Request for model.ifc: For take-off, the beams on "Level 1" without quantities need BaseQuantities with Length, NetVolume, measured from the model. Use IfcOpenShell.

First a look at what the model holds.

```python
import ifcopenshell
import ifcopenshell.util.element
import ifcopenshell.util.unit

model = ifcopenshell.open("model.ifc")
print(model.schema)
for unit_type in ("LENGTHUNIT", "AREAUNIT", "VOLUMEUNIT"):
    print(unit_type, ifcopenshell.util.unit.calculate_unit_scale(model, unit_type))
storey = next(s for s in model.by_type("IfcBuildingStorey") if s.Name == "Level 1")
beams = [e for e in ifcopenshell.util.element.get_decomposition(storey) if e.is_a("IfcBeam")]
for e in sorted(beams, key=lambda e: e.id()):
    print(e.id(), e.is_a(), e.Name, list(ifcopenshell.util.element.get_psets(e, qtos_only=True)), sep=" | ")
```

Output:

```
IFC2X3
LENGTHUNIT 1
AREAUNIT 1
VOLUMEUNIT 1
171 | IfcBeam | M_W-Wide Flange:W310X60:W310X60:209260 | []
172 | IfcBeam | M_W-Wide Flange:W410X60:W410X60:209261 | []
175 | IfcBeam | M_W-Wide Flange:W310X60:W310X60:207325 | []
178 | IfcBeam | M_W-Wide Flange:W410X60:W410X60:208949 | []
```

```python
import ifcopenshell
import ifcopenshell.api.pset
import ifcopenshell.geom
import ifcopenshell.util.element
import ifcopenshell.util.shape
import ifcopenshell.util.unit

model = ifcopenshell.open("model.ifc")
unit_scale = ifcopenshell.util.unit.calculate_unit_scale(model)
volume_scale = ifcopenshell.util.unit.calculate_unit_scale(model, "VOLUMEUNIT")
settings = ifcopenshell.geom.settings()

storey = next(s for s in model.by_type("IfcBuildingStorey") if s.Name == "Level 1")
beams = [e for e in ifcopenshell.util.element.get_decomposition(storey) if e.is_a("IfcBeam")]

for e in sorted(beams, key=lambda e: e.id()):
    if ifcopenshell.util.element.get_psets(e, qtos_only=True, should_inherit=False):
        continue
    # Geometry comes back in metres, in the element's own axes.
    shape = ifcopenshell.geom.create_shape(settings, e)
    values = {
        "Length": ifcopenshell.util.shape.get_max_xyz(shape.geometry) / unit_scale,
        "NetVolume": ifcopenshell.util.shape.get_volume(shape.geometry) / volume_scale,
    }
    qto = ifcopenshell.api.pset.add_qto(model, product=e, name="BaseQuantities")
    ifcopenshell.api.pset.edit_qto(model, qto=qto, properties=values)
    print(e.id(), {k: round(v, 3) for k, v in values.items()})

model.write("model_updated.ifc")
```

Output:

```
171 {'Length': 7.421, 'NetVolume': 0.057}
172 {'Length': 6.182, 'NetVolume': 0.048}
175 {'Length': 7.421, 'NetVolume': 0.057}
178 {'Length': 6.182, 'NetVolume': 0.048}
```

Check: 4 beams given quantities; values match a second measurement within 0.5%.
